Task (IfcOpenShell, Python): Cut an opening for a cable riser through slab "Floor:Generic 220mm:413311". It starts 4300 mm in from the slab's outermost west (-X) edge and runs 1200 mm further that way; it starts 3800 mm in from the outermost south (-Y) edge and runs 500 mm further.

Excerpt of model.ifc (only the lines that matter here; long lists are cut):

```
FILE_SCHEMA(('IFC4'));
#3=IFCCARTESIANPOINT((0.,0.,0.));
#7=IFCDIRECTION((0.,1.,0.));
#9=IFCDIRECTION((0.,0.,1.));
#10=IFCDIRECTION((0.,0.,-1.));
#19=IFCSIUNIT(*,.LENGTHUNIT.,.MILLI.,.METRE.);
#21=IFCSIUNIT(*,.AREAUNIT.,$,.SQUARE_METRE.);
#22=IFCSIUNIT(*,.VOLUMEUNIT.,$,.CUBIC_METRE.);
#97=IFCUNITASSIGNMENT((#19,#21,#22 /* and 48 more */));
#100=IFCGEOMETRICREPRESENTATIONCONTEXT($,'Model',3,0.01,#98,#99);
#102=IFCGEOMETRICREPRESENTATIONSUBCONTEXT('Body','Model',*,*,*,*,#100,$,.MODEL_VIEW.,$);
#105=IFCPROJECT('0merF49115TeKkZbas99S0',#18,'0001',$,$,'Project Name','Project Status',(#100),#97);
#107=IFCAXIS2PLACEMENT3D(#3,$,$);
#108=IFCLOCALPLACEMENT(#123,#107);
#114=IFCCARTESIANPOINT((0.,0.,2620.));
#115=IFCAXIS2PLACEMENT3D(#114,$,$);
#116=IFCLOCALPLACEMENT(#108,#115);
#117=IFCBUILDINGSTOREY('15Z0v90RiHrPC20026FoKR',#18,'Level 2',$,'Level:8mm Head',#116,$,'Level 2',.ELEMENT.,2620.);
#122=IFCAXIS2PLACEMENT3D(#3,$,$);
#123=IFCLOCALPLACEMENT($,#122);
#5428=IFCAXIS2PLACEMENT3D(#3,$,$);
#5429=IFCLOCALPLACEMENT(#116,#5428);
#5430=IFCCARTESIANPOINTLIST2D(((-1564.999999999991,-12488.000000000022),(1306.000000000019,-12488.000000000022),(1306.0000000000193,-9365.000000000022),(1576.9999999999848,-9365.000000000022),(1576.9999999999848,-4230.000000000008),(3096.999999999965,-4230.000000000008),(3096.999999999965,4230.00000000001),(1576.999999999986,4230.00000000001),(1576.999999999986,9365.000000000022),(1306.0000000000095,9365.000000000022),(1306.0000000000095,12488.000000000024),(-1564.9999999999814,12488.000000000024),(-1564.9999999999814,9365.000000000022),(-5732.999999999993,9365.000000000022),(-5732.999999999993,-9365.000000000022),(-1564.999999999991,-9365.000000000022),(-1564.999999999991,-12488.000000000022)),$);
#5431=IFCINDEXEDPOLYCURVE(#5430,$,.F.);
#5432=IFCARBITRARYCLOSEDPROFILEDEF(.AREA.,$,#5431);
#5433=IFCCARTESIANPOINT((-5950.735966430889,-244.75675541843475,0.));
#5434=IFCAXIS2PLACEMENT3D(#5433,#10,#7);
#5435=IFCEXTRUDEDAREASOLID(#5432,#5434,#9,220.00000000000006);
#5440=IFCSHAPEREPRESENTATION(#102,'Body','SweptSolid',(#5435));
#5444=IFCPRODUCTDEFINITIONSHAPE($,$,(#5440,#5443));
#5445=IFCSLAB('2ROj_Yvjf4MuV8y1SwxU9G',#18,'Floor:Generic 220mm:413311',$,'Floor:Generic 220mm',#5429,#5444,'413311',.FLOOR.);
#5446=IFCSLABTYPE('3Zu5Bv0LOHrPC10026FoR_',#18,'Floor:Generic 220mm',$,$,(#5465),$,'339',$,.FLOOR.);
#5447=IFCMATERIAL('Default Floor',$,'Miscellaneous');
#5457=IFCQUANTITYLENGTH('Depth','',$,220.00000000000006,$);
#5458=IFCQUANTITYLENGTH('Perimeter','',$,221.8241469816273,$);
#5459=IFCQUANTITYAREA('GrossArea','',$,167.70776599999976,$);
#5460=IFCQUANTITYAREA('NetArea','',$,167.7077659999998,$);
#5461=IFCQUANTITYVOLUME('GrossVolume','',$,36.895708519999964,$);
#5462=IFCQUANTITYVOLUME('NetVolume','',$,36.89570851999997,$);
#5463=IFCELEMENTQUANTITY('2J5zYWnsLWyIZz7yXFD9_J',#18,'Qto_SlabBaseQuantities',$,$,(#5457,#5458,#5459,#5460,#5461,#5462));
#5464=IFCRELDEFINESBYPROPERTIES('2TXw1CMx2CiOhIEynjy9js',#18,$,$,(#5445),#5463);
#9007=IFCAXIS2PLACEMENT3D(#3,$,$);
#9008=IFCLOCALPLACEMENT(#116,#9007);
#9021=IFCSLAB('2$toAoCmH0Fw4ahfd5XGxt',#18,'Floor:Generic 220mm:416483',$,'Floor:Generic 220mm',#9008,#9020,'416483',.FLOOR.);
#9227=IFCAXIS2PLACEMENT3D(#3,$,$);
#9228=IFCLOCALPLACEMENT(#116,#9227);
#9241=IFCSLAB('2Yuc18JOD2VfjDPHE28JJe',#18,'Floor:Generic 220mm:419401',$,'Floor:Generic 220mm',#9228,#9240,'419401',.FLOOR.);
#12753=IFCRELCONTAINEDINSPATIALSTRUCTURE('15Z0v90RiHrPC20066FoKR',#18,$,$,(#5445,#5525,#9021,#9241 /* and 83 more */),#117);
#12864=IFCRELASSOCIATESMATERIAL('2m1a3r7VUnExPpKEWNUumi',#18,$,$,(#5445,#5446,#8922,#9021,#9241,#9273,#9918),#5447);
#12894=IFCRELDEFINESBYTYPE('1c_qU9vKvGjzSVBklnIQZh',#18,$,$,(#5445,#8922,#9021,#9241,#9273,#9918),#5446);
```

```python
import numpy as np
import ifcopenshell
import ifcopenshell.api.feature
import ifcopenshell.api.geometry
import ifcopenshell.api.pset
import ifcopenshell.api.root
import ifcopenshell.geom
import ifcopenshell.util.element
import ifcopenshell.util.placement
import ifcopenshell.util.representation
import ifcopenshell.util.shape
import ifcopenshell.util.unit

model = ifcopenshell.open("model.ifc")
unit_scale = ifcopenshell.util.unit.calculate_unit_scale(model)
area_scale = ifcopenshell.util.unit.calculate_unit_scale(model, "AREAUNIT")
volume_scale = ifcopenshell.util.unit.calculate_unit_scale(model, "VOLUMEUNIT")
settings = ifcopenshell.geom.settings()


def volume(element):
    """Net volume in cubic metres, openings subtracted."""
    shape = ifcopenshell.geom.create_shape(settings, element)
    return ifcopenshell.util.shape.get_volume(shape.geometry)


slab = model.by_guid("2ROj_Yvjf4MuV8y1SwxU9G")
before = volume(slab)

# Extent in the slab's own axes, in metres. The edges named are its -X and -Y sides.
slab_shape = ifcopenshell.geom.create_shape(settings, slab)
vertices = ifcopenshell.util.shape.get_vertices(slab_shape.geometry)
x_min, y_min, bottom = vertices.min(axis=0)
top = vertices[:, 2].max()

opening = ifcopenshell.api.root.create_entity(model, ifc_class="IfcOpeningElement", name="Cable riser opening", predefined_type="OPENING")
context = ifcopenshell.util.representation.get_context(model, "Model", "Body", "MODEL_VIEW")
width, depth = 1.2, 0.5
outline = [(0.0, 0.0), (width, 0.0), (width, depth), (0.0, depth), (0.0, 0.0)]
# Overshoot both faces by 50 mm so the cut is clean.
shape = ifcopenshell.api.geometry.add_slab_representation(
    model, context=context, depth=top - bottom + 0.1, polyline=outline
)
ifcopenshell.api.geometry.assign_representation(model, product=opening, representation=shape)

matrix = ifcopenshell.util.placement.get_local_placement(slab.ObjectPlacement)
matrix[:, 3] = matrix @ np.append(np.array([x_min + 4.3, y_min + 3.8, bottom - 0.05]) / unit_scale, 1.0)
ifcopenshell.api.geometry.edit_object_placement(model, product=opening, matrix=matrix, is_si=False)
ifcopenshell.api.feature.add_feature(model, feature=opening, element=slab)

after = volume(slab)

# Update the slab's stored quantities.
qto = model.by_id(ifcopenshell.util.element.get_pset(slab, "Qto_SlabBaseQuantities", should_inherit=False)["id"])
ifcopenshell.api.pset.edit_qto(model, qto=qto, properties={
    "NetArea": after / (top - bottom) / area_scale,
    "NetVolume": after / volume_scale,
})

print(f"slab volume {before:.3f} -> {after:.3f} m3")

model.write("model_updated.ifc")
```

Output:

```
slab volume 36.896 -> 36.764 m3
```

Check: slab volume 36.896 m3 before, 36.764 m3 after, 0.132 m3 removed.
